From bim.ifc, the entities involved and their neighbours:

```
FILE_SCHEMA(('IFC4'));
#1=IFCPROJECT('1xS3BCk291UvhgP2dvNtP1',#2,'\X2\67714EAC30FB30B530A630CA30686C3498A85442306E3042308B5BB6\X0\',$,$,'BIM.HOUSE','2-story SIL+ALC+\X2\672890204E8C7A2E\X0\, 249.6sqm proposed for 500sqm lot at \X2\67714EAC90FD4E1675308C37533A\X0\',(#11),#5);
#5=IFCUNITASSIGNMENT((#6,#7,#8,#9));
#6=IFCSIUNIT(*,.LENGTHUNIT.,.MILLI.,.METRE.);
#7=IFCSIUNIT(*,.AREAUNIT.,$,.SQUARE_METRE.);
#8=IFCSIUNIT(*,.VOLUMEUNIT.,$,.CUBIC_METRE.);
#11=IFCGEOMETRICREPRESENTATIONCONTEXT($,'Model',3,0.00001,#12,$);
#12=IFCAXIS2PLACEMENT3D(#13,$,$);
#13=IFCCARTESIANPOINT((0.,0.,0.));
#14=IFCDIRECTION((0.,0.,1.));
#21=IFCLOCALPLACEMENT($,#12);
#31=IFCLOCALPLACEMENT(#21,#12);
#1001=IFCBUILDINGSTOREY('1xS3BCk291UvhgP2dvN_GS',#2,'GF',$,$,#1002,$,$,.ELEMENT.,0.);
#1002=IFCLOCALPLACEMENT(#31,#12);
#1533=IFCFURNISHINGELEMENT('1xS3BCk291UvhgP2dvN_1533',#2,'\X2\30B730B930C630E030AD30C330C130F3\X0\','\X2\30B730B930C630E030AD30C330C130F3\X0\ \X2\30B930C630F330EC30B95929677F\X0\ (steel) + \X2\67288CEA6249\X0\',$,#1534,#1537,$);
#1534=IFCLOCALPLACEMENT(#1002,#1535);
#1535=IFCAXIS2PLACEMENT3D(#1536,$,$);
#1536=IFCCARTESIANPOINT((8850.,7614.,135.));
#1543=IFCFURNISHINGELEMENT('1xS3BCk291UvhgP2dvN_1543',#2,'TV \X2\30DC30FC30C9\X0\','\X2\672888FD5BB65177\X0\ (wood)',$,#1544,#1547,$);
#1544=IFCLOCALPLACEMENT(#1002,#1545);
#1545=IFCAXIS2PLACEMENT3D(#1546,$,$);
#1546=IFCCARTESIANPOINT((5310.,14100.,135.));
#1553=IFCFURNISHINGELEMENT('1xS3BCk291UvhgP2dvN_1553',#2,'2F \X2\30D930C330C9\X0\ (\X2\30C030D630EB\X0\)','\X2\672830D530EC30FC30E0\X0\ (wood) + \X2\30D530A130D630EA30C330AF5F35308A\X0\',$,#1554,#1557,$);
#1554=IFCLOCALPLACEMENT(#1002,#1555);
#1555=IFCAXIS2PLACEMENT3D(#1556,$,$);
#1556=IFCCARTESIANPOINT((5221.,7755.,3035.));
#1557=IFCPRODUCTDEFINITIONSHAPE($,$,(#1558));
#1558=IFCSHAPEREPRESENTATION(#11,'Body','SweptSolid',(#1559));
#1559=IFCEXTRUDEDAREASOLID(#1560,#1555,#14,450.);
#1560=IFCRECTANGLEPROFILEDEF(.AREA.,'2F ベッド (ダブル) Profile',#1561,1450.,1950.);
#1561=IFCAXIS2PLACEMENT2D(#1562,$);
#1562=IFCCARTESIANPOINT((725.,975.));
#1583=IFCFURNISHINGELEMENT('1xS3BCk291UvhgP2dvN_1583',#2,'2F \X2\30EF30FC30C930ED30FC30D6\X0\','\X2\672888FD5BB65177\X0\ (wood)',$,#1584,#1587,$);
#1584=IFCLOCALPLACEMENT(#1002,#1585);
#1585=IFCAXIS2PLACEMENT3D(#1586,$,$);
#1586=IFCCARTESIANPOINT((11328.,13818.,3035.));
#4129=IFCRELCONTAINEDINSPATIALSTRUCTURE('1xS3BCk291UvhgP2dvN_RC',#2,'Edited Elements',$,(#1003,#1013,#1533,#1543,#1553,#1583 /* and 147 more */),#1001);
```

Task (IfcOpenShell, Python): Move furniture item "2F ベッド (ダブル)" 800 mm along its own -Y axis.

```python
import ifcopenshell
import ifcopenshell.api.geometry
import ifcopenshell.util.placement
import ifcopenshell.util.unit

model = ifcopenshell.open("bim.ifc")
unit_scale = ifcopenshell.util.unit.calculate_unit_scale(model)

item = model.by_guid("1xS3BCk291UvhgP2dvN_1553")
matrix = ifcopenshell.util.placement.get_local_placement(item.ObjectPlacement)
matrix[:3, 3] -= matrix[:3, 1] * 0.8 / unit_scale
ifcopenshell.api.geometry.edit_object_placement(model, product=item, matrix=matrix, is_si=False)

print(ifcopenshell.util.placement.get_local_placement(item.ObjectPlacement).round(3) + 0.0)

model.write("bim_updated.ifc")
```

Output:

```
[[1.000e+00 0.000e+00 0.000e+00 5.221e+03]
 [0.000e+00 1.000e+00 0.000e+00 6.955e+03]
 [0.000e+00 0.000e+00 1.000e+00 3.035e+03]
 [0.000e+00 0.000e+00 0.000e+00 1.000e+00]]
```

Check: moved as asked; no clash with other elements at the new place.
